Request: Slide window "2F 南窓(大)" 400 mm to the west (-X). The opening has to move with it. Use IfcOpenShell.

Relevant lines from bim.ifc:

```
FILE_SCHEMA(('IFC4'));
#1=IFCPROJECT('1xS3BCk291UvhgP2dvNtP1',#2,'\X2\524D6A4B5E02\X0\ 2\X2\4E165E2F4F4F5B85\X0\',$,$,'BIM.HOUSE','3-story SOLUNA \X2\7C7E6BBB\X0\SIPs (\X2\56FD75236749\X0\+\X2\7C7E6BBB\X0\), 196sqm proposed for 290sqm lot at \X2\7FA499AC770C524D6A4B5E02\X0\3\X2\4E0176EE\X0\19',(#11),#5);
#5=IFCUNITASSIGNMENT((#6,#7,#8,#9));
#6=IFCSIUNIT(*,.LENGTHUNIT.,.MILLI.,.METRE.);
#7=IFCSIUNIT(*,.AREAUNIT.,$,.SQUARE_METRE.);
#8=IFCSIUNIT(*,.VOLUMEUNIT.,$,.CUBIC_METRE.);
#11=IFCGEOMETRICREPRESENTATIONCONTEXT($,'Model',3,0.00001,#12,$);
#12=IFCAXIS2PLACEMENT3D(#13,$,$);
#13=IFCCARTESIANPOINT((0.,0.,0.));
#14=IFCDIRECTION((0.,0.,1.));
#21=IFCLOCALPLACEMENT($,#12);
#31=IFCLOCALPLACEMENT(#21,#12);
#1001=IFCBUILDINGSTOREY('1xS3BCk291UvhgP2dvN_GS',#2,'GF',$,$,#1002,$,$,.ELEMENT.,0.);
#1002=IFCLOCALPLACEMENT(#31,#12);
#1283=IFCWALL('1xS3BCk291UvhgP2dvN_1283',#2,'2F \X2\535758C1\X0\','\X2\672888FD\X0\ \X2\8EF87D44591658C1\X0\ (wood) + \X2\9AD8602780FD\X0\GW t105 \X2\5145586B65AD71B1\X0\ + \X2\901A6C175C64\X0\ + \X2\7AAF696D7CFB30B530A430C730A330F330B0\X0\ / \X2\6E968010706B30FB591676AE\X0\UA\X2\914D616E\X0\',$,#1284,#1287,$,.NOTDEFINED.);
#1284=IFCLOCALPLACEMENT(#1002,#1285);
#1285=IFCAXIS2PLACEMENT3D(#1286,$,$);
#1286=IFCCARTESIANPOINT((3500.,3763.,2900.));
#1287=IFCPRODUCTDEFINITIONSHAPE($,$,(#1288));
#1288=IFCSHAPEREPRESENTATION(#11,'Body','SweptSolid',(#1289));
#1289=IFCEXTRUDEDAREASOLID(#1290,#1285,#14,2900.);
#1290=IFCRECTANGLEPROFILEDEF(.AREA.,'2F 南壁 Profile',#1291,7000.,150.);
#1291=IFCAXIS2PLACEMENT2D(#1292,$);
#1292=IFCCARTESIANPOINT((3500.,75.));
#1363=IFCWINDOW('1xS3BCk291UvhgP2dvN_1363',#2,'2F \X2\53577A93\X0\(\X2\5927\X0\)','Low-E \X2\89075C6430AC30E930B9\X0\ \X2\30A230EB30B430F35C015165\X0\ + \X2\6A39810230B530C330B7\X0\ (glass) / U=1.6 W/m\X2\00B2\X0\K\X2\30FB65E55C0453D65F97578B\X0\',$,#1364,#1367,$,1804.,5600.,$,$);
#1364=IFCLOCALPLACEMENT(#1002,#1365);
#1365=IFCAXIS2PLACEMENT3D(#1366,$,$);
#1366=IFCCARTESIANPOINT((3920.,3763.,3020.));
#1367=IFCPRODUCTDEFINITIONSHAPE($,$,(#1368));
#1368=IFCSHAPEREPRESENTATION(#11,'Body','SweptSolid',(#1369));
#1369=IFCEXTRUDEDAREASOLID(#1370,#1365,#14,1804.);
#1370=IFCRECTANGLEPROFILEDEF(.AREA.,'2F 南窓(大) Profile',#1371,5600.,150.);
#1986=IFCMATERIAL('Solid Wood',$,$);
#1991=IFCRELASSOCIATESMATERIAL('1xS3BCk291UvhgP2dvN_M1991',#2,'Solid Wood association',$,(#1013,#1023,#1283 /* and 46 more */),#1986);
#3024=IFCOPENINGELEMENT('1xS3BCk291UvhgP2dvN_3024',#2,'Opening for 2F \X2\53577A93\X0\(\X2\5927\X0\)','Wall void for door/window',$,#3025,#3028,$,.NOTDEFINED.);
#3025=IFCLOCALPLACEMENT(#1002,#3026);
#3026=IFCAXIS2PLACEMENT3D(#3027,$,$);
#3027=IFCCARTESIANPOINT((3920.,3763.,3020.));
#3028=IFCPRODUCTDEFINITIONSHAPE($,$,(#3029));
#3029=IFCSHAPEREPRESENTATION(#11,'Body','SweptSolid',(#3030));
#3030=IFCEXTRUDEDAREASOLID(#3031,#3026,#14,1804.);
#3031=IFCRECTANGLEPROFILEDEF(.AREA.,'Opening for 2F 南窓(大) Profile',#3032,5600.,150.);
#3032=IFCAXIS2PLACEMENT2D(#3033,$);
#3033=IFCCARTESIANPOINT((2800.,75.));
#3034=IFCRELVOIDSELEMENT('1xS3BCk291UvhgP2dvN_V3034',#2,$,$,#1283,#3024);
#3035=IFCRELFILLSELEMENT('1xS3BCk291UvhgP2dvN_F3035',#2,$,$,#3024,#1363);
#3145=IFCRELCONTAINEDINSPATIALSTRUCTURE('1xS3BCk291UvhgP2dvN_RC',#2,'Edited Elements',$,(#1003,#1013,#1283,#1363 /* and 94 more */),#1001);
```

```python
import ifcopenshell
import ifcopenshell.api.geometry
import ifcopenshell.util.placement
import ifcopenshell.util.unit

model = ifcopenshell.open("bim.ifc")
unit_scale = ifcopenshell.util.unit.calculate_unit_scale(model)

window = model.by_guid("1xS3BCk291UvhgP2dvN_1363")
opening = window.FillsVoids[0].RelatingOpeningElement
wall = opening.VoidsElements[0].RelatingBuildingElement

wall_matrix = ifcopenshell.util.placement.get_local_placement(wall.ObjectPlacement)
shift = wall_matrix[:3, 0] * -0.4 / unit_scale
before = ifcopenshell.util.placement.get_local_placement(window.ObjectPlacement)[:3, 3].copy()

# The window is not placed relative to its opening, so move both.
for product in (opening, window):
    matrix = ifcopenshell.util.placement.get_local_placement(product.ObjectPlacement)
    matrix[:3, 3] += shift
    ifcopenshell.api.geometry.edit_object_placement(model, product=product, matrix=matrix, is_si=False)

after = ifcopenshell.util.placement.get_local_placement(window.ObjectPlacement)[:3, 3]
print("window moved by", (after - before).round(3) + 0.0)

model.write("bim_edited.ifc")
```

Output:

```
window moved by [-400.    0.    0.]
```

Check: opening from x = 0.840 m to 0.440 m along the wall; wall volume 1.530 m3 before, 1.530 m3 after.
